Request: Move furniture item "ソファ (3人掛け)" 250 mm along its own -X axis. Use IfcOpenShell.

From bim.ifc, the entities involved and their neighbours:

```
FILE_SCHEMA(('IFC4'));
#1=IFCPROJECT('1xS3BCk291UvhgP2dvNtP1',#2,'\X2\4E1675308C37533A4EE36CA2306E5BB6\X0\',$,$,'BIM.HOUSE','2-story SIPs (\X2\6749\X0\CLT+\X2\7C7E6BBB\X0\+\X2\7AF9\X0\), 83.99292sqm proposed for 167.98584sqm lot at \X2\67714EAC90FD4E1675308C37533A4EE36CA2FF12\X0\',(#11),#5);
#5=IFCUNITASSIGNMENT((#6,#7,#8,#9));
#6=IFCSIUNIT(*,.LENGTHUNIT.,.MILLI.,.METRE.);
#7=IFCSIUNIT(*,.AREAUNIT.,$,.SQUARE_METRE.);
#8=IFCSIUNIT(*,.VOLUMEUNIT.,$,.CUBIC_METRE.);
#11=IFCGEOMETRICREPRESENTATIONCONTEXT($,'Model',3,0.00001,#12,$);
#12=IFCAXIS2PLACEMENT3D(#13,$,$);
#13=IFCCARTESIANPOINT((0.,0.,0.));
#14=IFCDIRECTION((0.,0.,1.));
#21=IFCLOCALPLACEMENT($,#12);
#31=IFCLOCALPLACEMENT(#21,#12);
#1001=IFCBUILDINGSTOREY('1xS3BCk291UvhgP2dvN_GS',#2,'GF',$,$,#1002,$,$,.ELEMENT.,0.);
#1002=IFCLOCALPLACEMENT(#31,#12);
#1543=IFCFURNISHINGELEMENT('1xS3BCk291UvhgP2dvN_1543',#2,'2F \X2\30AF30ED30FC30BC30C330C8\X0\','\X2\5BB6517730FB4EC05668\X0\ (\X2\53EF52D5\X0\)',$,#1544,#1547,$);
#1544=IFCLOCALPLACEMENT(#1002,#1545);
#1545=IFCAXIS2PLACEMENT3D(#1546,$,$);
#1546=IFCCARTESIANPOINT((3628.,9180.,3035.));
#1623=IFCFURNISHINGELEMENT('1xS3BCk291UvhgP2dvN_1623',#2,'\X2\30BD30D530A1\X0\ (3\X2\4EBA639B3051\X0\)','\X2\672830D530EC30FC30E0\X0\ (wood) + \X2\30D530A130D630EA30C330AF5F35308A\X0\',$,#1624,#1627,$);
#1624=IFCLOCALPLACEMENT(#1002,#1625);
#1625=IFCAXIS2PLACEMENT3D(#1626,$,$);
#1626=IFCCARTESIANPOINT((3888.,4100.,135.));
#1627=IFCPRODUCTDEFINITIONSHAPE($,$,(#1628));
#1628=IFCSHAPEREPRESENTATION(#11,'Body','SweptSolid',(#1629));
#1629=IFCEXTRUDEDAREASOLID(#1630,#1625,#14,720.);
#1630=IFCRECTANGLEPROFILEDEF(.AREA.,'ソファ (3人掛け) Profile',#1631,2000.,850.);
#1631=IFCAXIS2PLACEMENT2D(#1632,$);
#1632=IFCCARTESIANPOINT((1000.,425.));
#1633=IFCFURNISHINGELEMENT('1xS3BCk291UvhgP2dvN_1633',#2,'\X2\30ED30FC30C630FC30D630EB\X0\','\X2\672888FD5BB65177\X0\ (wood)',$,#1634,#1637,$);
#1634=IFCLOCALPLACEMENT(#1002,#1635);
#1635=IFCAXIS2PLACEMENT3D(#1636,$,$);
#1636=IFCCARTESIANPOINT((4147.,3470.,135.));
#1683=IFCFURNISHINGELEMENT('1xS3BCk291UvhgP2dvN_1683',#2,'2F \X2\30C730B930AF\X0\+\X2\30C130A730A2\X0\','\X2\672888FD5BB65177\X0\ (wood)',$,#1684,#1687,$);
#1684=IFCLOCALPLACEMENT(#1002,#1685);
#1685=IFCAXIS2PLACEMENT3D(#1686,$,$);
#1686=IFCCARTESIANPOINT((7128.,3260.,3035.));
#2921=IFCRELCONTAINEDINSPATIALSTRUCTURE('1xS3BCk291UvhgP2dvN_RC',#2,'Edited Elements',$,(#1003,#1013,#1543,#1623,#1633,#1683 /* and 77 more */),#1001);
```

```python
import ifcopenshell
import ifcopenshell.api.geometry
import ifcopenshell.util.placement
import ifcopenshell.util.unit

model = ifcopenshell.open("bim.ifc")
unit_scale = ifcopenshell.util.unit.calculate_unit_scale(model)

item = model.by_guid("1xS3BCk291UvhgP2dvN_1623")
matrix = ifcopenshell.util.placement.get_local_placement(item.ObjectPlacement)
matrix[:3, 3] -= matrix[:3, 0] * 0.25 / unit_scale
ifcopenshell.api.geometry.edit_object_placement(model, product=item, matrix=matrix, is_si=False)

print(ifcopenshell.util.placement.get_local_placement(item.ObjectPlacement).round(3) + 0.0)

model.write("bim_updated.ifc")
```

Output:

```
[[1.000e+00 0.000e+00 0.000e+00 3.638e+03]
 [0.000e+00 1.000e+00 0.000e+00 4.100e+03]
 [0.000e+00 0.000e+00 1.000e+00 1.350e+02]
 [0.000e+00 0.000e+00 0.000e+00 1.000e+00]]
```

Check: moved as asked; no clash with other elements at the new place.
